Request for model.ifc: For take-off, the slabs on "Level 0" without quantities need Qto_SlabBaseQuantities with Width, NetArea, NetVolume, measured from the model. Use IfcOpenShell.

First a look at what the model holds.

```python
import ifcopenshell
import ifcopenshell.util.element
import ifcopenshell.util.unit

model = ifcopenshell.open("model.ifc")
print(model.schema)
for unit_type in ("LENGTHUNIT", "AREAUNIT", "VOLUMEUNIT"):
    print(unit_type, ifcopenshell.util.unit.calculate_unit_scale(model, unit_type))
storey = next(s for s in model.by_type("IfcBuildingStorey") if s.Name == "Level 0")
slabs = [e for e in ifcopenshell.util.element.get_decomposition(storey) if e.is_a("IfcSlab")]
for e in sorted(slabs, key=lambda e: e.id()):
    print(e.id(), e.is_a(), e.Name, list(ifcopenshell.util.element.get_psets(e, qtos_only=True)), sep=" | ")
```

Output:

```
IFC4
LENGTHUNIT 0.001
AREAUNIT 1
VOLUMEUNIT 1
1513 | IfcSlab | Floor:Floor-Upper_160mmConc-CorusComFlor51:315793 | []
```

```python
import ifcopenshell
import ifcopenshell.api.pset
import ifcopenshell.geom
import ifcopenshell.util.element
import ifcopenshell.util.shape
import ifcopenshell.util.unit

model = ifcopenshell.open("model.ifc")
unit_scale = ifcopenshell.util.unit.calculate_unit_scale(model)
area_scale = ifcopenshell.util.unit.calculate_unit_scale(model, "AREAUNIT")
volume_scale = ifcopenshell.util.unit.calculate_unit_scale(model, "VOLUMEUNIT")
settings = ifcopenshell.geom.settings()

storey = next(s for s in model.by_type("IfcBuildingStorey") if s.Name == "Level 0")
slabs = [e for e in ifcopenshell.util.element.get_decomposition(storey) if e.is_a("IfcSlab")]

for e in sorted(slabs, key=lambda e: e.id()):
    if ifcopenshell.util.element.get_psets(e, qtos_only=True, should_inherit=False):
        continue
    # Geometry comes back in metres, in the element's own axes.
    shape = ifcopenshell.geom.create_shape(settings, e)
    values = {
        "Width": ifcopenshell.util.shape.get_z(shape.geometry) / unit_scale,
        "NetArea": ifcopenshell.util.shape.get_footprint_area(shape.geometry) / area_scale,
        "NetVolume": ifcopenshell.util.shape.get_volume(shape.geometry) / volume_scale,
    }
    qto = ifcopenshell.api.pset.add_qto(model, product=e, name="Qto_SlabBaseQuantities")
    ifcopenshell.api.pset.edit_qto(model, qto=qto, properties=values)
    print(e.id(), {k: round(v, 3) for k, v in values.items()})

model.write("model-out.ifc")
```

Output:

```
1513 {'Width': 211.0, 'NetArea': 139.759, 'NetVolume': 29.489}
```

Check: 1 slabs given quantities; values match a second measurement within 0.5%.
